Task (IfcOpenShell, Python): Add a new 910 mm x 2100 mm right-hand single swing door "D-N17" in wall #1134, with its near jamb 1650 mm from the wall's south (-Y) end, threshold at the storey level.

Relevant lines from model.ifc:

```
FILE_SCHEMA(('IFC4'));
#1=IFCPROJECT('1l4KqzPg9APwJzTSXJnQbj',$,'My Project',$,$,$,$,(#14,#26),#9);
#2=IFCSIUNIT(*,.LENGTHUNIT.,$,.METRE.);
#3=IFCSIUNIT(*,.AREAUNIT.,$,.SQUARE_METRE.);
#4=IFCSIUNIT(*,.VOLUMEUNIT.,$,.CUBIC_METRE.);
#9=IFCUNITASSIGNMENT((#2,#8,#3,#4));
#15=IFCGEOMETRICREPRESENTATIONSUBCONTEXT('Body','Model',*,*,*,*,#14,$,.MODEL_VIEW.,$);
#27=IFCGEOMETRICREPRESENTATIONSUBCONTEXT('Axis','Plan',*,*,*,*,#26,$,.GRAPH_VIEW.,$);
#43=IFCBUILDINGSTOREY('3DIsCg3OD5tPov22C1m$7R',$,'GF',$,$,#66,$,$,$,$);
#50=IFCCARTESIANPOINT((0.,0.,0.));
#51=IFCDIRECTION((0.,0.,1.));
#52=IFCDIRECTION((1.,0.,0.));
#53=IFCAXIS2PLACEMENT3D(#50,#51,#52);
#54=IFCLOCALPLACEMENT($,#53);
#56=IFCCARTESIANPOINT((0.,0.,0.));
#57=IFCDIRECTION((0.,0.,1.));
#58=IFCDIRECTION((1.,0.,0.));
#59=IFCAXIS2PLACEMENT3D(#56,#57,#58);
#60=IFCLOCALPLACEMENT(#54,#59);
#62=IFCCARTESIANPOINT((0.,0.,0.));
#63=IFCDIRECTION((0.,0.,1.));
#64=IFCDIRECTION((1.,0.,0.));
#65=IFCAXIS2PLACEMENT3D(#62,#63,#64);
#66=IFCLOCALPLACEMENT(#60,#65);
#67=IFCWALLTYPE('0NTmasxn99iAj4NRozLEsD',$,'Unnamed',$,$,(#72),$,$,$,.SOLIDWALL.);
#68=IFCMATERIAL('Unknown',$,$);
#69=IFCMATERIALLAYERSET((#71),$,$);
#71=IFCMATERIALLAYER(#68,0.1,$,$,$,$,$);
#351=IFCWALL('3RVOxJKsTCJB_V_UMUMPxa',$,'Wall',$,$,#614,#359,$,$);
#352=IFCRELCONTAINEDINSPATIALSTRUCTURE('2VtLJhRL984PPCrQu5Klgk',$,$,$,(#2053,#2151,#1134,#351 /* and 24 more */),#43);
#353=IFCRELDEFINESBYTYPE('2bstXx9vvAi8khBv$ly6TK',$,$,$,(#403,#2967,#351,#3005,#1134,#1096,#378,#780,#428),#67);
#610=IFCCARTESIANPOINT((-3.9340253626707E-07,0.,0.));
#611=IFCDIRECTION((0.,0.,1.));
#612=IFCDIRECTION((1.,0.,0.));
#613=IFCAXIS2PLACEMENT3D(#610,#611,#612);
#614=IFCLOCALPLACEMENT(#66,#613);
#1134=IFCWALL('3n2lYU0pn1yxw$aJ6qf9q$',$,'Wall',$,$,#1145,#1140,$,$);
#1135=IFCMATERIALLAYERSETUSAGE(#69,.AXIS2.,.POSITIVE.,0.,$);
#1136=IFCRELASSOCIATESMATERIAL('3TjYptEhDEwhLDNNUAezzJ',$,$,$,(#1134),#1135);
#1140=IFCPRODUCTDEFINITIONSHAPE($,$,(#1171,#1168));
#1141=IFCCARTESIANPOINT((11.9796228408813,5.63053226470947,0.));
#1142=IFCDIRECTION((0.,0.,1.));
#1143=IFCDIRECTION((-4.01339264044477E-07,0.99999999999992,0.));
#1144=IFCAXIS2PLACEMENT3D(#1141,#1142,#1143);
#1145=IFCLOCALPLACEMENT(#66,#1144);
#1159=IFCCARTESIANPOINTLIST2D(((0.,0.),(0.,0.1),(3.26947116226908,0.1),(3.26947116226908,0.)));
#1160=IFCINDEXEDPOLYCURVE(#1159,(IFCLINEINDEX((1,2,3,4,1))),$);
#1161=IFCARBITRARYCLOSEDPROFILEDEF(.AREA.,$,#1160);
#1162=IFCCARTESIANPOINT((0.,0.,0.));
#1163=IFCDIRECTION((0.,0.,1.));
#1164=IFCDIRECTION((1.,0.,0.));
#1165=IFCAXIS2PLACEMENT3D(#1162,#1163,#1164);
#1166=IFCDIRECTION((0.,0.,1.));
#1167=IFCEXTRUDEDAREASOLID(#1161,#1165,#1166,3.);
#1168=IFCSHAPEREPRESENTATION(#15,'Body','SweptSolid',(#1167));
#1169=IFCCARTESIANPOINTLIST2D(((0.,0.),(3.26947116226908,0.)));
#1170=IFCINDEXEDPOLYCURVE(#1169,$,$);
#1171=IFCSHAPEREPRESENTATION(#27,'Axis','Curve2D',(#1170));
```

```python
import numpy as np
import ifcopenshell
import ifcopenshell.api.feature
import ifcopenshell.api.geometry
import ifcopenshell.api.root
import ifcopenshell.api.spatial
import ifcopenshell.geom
import ifcopenshell.util.element
import ifcopenshell.util.placement
import ifcopenshell.util.representation
import ifcopenshell.util.shape
import ifcopenshell.util.unit

model = ifcopenshell.open("model.ifc")
unit_scale = ifcopenshell.util.unit.calculate_unit_scale(model)
settings = ifcopenshell.geom.settings()


def volume(element):
    """Net volume in cubic metres, openings subtracted."""
    shape = ifcopenshell.geom.create_shape(settings, element)
    return ifcopenshell.util.shape.get_volume(shape.geometry)


wall = model.by_guid("3n2lYU0pn1yxw$aJ6qf9q$")
storey = ifcopenshell.util.element.get_container(wall, ifc_class="IfcBuildingStorey")
context = ifcopenshell.util.representation.get_context(model, "Model", "Body", "MODEL_VIEW")
before = volume(wall)

width, height, from_end, sill = 0.91, 2.1, 1.65, 0.0  # metres

# The wall runs along its own X axis, and the end named is its -X end.
wall_shape = ifcopenshell.geom.create_shape(settings, wall)
x, y, z = ifcopenshell.util.shape.get_vertices(wall_shape.geometry).T
start = x.min() + from_end
face, thickness = float(y.min()), float(y.max() - y.min())
wall_matrix = ifcopenshell.util.placement.get_local_placement(wall.ObjectPlacement)
level = ifcopenshell.util.placement.get_local_placement(storey.ObjectPlacement)[2, 3]


def in_wall(x, y):
    """Placement at x, y metres in the wall's axes, at sill height."""
    matrix = wall_matrix.copy()
    matrix[:, 3] = wall_matrix @ np.array([x / unit_scale, y / unit_scale, 0.0, 1.0])
    matrix[2, 3] = level + sill / unit_scale
    return matrix


# Opening: a box that overshoots both wall faces by 50 mm.
opening = ifcopenshell.api.root.create_entity(model, ifc_class="IfcOpeningElement", predefined_type="OPENING")
box = ifcopenshell.api.geometry.add_wall_representation(
    model, context=context, length=width, height=height, thickness=thickness + 0.1
)
ifcopenshell.api.geometry.assign_representation(model, product=opening, representation=box)
ifcopenshell.api.geometry.edit_object_placement(model, product=opening, matrix=in_wall(start, face - 0.05), is_si=False)
ifcopenshell.api.feature.add_feature(model, feature=opening, element=wall)

door = ifcopenshell.api.root.create_entity(model, ifc_class="IfcDoor", name="D-N17", predefined_type="DOOR")
door.OverallWidth, door.OverallHeight = width / unit_scale, height / unit_scale
door.OperationType = "SINGLE_SWING_RIGHT"
body = ifcopenshell.api.geometry.add_door_representation(
    model,
    context=context,
    overall_width=door.OverallWidth,
    overall_height=door.OverallHeight,
    operation_type="SINGLE_SWING_RIGHT",
    lining_properties={"LiningDepth": thickness / unit_scale, "ThresholdDepth": thickness / unit_scale},
)
ifcopenshell.api.geometry.assign_representation(model, product=door, representation=body)
ifcopenshell.api.spatial.assign_container(model, products=[door], relating_structure=storey)
ifcopenshell.api.feature.add_filling(model, opening=opening, element=door)

# The lining spans the wall, so the door starts at the wall face.
ifcopenshell.api.geometry.edit_object_placement(model, product=door, matrix=in_wall(start, face), is_si=False)

after = volume(wall)

print(f"wall volume {before:.3f} -> {after:.3f} m3")

model.write("model_edited.ifc")
```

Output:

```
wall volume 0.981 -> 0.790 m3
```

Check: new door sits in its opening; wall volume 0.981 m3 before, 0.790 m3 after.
